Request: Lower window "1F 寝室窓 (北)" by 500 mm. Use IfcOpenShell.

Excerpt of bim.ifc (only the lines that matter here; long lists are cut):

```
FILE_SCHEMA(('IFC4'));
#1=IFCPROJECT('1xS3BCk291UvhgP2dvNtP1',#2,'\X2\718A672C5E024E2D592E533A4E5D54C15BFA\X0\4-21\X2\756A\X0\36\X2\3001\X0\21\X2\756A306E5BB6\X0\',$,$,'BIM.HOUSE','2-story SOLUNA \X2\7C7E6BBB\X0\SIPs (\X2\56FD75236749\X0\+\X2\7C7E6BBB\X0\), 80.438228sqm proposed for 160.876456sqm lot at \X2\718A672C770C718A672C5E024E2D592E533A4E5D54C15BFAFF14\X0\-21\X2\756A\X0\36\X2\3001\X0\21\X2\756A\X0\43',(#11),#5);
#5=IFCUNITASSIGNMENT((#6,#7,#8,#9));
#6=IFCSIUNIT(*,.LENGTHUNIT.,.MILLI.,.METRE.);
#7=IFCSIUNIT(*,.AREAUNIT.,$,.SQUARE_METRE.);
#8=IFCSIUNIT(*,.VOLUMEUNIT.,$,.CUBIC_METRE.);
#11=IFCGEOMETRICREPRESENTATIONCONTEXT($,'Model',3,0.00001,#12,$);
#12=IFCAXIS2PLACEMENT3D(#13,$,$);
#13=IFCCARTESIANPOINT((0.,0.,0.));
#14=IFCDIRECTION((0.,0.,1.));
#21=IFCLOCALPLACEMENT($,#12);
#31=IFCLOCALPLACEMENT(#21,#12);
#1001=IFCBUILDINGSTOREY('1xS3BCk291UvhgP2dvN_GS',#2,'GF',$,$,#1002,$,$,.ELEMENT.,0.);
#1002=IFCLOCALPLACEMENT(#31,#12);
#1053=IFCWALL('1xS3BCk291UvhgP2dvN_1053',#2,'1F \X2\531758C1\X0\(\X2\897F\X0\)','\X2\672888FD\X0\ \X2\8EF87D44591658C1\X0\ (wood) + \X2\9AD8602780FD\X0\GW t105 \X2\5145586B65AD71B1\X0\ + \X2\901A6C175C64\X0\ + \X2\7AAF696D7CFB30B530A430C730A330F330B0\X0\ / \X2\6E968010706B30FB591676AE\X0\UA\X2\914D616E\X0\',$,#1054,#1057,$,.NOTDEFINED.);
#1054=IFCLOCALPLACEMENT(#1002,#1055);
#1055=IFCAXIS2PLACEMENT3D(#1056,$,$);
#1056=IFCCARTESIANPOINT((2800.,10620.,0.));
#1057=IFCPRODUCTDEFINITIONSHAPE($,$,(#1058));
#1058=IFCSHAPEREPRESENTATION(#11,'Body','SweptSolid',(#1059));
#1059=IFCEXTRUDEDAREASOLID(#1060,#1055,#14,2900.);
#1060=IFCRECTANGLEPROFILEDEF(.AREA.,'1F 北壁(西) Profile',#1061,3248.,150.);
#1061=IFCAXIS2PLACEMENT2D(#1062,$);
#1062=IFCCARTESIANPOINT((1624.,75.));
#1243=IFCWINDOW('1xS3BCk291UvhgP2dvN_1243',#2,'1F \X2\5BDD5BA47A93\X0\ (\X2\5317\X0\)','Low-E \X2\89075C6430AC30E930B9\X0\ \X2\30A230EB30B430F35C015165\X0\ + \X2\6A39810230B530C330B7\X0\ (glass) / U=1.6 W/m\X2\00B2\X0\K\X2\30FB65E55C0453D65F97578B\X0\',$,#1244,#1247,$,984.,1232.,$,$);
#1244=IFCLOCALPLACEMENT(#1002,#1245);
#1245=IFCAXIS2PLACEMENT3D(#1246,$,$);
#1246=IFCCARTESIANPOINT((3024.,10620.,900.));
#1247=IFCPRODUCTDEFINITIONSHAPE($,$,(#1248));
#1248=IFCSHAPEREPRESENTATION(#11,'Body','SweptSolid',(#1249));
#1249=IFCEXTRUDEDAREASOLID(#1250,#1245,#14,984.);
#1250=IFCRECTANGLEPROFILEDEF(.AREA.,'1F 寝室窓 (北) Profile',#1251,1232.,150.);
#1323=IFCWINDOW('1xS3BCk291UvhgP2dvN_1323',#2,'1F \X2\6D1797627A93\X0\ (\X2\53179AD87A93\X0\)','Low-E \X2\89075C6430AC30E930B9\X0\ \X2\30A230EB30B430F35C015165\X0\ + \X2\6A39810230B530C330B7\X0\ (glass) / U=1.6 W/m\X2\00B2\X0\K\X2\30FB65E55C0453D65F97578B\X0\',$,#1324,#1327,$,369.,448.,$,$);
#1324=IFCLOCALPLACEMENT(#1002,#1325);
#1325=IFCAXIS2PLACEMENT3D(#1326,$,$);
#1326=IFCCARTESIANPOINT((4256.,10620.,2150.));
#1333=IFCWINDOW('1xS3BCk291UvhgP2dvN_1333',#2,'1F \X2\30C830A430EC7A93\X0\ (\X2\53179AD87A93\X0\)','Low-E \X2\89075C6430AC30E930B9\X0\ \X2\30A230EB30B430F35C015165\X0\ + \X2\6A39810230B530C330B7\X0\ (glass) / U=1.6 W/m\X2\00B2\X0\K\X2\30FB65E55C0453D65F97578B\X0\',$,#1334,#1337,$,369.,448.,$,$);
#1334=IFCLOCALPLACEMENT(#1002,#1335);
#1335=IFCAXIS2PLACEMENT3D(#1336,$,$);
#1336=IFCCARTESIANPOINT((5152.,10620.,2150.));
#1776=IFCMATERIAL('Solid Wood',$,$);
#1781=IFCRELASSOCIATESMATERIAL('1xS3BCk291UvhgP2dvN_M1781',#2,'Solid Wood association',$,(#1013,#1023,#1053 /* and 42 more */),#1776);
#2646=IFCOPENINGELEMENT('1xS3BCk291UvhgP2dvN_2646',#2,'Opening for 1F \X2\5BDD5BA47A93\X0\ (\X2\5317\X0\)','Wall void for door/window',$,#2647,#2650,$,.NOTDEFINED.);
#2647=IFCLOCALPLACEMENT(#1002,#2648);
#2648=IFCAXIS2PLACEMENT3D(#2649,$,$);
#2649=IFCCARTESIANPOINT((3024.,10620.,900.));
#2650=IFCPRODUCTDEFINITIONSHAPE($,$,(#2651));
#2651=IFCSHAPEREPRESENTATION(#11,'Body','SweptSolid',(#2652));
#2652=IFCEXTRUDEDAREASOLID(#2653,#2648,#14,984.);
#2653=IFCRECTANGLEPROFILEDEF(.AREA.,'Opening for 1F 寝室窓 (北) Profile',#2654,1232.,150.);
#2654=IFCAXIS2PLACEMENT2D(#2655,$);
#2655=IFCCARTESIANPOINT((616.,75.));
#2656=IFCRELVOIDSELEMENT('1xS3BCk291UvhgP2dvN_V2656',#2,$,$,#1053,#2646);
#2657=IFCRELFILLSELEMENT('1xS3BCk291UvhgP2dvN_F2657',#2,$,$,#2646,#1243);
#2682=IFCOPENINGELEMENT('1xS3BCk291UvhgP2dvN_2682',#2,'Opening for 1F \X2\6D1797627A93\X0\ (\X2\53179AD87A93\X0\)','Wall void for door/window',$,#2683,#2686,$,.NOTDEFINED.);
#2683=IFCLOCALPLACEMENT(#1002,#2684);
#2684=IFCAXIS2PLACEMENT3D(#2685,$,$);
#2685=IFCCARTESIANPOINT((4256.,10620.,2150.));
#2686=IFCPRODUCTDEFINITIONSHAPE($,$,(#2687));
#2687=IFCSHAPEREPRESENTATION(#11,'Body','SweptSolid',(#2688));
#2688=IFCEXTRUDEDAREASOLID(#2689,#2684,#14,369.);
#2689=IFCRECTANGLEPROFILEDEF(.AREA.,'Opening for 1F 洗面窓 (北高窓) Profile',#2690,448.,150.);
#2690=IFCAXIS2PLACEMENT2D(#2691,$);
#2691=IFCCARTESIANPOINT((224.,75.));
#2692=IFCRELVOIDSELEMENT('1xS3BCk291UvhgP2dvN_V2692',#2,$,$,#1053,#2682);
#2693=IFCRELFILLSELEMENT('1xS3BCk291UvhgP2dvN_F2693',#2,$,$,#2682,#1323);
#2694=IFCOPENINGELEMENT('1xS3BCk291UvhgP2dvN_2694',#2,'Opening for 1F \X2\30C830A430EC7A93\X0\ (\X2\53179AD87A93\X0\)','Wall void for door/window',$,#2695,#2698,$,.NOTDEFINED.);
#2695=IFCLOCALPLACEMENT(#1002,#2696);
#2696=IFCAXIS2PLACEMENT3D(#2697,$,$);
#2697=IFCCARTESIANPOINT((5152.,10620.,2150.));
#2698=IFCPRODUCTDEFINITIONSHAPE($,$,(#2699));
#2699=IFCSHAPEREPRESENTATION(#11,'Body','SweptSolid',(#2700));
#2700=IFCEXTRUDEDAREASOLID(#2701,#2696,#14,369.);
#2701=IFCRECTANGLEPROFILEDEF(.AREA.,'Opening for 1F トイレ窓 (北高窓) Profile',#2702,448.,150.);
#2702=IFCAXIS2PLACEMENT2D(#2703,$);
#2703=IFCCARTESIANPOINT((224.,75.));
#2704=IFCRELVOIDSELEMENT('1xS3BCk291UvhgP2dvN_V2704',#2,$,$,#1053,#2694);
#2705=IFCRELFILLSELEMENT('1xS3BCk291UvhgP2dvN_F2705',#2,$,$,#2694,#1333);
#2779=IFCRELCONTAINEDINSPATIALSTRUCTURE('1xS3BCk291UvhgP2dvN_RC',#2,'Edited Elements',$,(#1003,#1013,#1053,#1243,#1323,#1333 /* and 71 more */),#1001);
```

```python
import numpy as np
import ifcopenshell
import ifcopenshell.api.geometry
import ifcopenshell.util.placement
import ifcopenshell.util.unit

model = ifcopenshell.open("bim.ifc")
unit_scale = ifcopenshell.util.unit.calculate_unit_scale(model)

window = model.by_guid("1xS3BCk291UvhgP2dvN_1243")
opening = window.FillsVoids[0].RelatingOpeningElement
dz = -0.5 / unit_scale

shift = np.array([0.0, 0.0, dz])
# The window is not placed relative to its opening, so move both.
for product in (opening, window):
    matrix = ifcopenshell.util.placement.get_local_placement(product.ObjectPlacement)
    matrix[:3, 3] += shift
    ifcopenshell.api.geometry.edit_object_placement(model, product=product, matrix=matrix, is_si=False)

print(f"moved by {dz * unit_scale:+.3f} m")

model.write("bim-out.ifc")
```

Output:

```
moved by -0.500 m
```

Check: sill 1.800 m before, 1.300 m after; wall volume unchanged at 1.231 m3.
